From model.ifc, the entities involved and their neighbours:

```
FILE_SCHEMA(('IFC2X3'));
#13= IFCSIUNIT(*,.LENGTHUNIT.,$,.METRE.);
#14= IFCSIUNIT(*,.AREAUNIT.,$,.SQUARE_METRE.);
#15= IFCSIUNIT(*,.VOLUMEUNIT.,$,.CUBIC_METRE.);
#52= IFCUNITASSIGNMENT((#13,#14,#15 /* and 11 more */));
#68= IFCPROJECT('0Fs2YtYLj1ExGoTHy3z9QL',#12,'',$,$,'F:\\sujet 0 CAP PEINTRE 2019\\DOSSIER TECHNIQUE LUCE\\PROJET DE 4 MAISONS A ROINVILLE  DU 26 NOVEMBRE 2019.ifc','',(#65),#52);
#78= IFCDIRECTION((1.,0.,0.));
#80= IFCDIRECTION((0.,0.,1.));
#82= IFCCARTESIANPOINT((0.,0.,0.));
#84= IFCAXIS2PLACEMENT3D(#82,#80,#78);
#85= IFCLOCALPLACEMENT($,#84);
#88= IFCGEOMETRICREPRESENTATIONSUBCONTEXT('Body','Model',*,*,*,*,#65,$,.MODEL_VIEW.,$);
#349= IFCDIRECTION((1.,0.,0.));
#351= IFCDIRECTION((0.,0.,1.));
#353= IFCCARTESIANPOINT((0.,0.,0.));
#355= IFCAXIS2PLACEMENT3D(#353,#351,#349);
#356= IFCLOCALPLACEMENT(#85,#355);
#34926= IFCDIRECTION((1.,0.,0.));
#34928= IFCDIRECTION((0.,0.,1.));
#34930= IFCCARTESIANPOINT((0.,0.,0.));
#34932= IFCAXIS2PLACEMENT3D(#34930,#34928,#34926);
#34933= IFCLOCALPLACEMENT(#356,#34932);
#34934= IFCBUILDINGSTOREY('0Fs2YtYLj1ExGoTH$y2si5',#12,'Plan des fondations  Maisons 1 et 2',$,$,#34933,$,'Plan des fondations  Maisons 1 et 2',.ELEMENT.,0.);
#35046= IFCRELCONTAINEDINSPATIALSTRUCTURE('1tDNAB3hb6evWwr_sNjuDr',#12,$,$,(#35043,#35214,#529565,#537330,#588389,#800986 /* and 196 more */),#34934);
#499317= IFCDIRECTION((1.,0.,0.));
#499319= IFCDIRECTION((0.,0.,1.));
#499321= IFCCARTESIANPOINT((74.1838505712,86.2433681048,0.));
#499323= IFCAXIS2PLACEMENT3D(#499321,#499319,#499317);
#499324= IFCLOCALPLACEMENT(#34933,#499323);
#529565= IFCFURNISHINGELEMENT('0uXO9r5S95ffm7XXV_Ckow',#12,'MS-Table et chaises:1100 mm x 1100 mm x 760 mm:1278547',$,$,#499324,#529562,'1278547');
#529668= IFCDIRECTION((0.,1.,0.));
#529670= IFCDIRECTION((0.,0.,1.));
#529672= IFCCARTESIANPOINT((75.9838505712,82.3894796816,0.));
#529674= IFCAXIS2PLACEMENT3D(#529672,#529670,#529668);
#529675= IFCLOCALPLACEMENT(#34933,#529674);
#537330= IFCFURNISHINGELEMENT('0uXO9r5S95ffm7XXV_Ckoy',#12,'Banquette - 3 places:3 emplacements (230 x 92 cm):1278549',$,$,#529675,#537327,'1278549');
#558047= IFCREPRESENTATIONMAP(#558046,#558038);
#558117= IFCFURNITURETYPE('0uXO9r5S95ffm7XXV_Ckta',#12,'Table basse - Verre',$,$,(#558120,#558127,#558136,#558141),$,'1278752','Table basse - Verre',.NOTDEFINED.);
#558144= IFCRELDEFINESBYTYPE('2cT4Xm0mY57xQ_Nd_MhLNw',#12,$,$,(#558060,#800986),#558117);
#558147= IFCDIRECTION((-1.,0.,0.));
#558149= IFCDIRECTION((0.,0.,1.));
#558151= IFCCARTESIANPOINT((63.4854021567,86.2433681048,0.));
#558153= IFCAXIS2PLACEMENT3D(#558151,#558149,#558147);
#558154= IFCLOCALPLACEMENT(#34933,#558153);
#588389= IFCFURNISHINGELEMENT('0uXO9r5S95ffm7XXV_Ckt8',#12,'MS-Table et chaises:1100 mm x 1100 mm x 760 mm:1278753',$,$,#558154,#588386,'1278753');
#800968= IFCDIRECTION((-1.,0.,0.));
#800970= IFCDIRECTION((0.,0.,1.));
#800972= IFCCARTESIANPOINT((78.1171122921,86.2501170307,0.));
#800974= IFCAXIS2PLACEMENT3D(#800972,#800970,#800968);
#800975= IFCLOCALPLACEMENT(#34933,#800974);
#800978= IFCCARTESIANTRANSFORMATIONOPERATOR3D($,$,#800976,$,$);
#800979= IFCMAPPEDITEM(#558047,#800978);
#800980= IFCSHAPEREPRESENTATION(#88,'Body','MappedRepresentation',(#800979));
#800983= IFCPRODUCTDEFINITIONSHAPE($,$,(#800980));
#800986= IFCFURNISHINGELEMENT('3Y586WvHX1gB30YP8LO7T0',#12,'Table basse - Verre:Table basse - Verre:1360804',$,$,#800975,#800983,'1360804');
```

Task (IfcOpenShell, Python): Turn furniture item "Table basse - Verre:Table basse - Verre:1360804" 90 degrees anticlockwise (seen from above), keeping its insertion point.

```python
import ifcopenshell
import ifcopenshell.api.geometry
import ifcopenshell.util.placement

model = ifcopenshell.open("model.ifc")

item = model.by_guid("3Y586WvHX1gB30YP8LO7T0")
matrix = ifcopenshell.util.placement.get_local_placement(item.ObjectPlacement)
matrix = matrix @ ifcopenshell.util.placement.rotation(90, "Z")
ifcopenshell.api.geometry.edit_object_placement(model, product=item, matrix=matrix, is_si=False)

print(ifcopenshell.util.placement.get_local_placement(item.ObjectPlacement).round(3) + 0.0)

model.write("model_rev.ifc")
```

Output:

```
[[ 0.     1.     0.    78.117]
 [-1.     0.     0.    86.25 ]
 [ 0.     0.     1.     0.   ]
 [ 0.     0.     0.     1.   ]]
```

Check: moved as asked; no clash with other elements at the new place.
